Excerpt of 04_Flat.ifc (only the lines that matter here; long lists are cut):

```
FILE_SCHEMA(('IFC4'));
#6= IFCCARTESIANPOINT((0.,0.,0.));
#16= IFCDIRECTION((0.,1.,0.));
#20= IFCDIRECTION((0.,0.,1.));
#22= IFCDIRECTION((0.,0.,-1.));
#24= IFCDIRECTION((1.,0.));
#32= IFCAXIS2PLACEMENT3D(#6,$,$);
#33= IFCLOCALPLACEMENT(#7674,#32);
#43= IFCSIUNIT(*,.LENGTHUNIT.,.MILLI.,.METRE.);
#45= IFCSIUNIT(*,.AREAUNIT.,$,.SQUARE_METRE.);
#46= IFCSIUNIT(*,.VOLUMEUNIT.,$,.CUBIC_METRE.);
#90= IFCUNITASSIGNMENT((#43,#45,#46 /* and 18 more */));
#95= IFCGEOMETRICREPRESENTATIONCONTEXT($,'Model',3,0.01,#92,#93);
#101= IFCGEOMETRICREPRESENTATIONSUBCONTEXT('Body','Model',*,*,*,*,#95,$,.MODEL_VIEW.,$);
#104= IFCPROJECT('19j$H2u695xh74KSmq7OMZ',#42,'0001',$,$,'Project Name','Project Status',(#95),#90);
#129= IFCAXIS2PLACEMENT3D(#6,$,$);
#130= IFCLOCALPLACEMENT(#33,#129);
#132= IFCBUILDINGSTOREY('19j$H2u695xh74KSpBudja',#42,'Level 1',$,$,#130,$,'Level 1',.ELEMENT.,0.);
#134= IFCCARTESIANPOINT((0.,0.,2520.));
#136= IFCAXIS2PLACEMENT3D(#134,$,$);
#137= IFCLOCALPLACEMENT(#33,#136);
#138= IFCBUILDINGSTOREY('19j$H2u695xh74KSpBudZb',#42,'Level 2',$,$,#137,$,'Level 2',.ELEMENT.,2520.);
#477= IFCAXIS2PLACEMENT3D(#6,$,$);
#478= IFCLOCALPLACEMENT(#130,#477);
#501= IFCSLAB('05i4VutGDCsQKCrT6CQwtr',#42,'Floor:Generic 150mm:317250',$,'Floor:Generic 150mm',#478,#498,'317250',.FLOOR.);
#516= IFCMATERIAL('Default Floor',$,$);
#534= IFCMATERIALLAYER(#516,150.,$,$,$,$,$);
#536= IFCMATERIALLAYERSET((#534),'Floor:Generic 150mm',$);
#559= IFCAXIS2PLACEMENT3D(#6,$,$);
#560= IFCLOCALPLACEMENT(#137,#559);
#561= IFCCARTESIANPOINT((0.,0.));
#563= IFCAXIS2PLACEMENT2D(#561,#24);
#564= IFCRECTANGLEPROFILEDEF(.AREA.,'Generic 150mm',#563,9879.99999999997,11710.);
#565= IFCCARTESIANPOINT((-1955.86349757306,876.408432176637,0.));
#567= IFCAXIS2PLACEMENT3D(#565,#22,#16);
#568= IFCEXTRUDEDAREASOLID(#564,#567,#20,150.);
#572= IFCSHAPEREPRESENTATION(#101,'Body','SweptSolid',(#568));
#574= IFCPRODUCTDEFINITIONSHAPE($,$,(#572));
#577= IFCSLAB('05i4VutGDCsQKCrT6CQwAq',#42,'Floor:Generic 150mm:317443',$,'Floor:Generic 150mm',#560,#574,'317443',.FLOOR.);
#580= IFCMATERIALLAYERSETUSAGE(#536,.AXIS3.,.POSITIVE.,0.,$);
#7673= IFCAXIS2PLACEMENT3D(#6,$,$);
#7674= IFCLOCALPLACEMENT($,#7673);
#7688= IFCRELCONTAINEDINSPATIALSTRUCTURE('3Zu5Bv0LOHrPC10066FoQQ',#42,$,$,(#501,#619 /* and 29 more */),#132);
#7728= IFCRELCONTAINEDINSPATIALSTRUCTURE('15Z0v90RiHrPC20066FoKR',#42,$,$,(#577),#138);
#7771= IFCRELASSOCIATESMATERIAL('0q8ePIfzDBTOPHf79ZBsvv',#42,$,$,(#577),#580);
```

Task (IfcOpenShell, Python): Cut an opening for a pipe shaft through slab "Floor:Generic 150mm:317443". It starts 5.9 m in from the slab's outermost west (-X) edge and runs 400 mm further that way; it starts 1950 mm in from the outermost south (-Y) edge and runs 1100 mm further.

```python
import numpy as np
import ifcopenshell
import ifcopenshell.api.feature
import ifcopenshell.api.geometry
import ifcopenshell.api.root
import ifcopenshell.geom
import ifcopenshell.util.placement
import ifcopenshell.util.representation
import ifcopenshell.util.shape
import ifcopenshell.util.unit

model = ifcopenshell.open("04_Flat.ifc")
unit_scale = ifcopenshell.util.unit.calculate_unit_scale(model)
settings = ifcopenshell.geom.settings()


def volume(element):
    """Net volume in cubic metres, openings subtracted."""
    shape = ifcopenshell.geom.create_shape(settings, element)
    return ifcopenshell.util.shape.get_volume(shape.geometry)


slab = model.by_guid("05i4VutGDCsQKCrT6CQwAq")
before = volume(slab)

# Extent in the slab's own axes, in metres. The edges named are its -X and -Y sides.
slab_shape = ifcopenshell.geom.create_shape(settings, slab)
vertices = ifcopenshell.util.shape.get_vertices(slab_shape.geometry)
x_min, y_min, bottom = vertices.min(axis=0)
top = vertices[:, 2].max()

opening = ifcopenshell.api.root.create_entity(model, ifc_class="IfcOpeningElement", name="Pipe shaft opening", predefined_type="OPENING")
context = ifcopenshell.util.representation.get_context(model, "Model", "Body", "MODEL_VIEW")
width, depth = 0.4, 1.1
outline = [(0.0, 0.0), (width, 0.0), (width, depth), (0.0, depth), (0.0, 0.0)]
# Overshoot both faces by 50 mm so the cut is clean.
shape = ifcopenshell.api.geometry.add_slab_representation(
    model, context=context, depth=top - bottom + 0.1, polyline=outline
)
ifcopenshell.api.geometry.assign_representation(model, product=opening, representation=shape)

matrix = ifcopenshell.util.placement.get_local_placement(slab.ObjectPlacement)
matrix[:, 3] = matrix @ np.append(np.array([x_min + 5.9, y_min + 1.95, bottom - 0.05]) / unit_scale, 1.0)
ifcopenshell.api.geometry.edit_object_placement(model, product=opening, matrix=matrix, is_si=False)
ifcopenshell.api.feature.add_feature(model, feature=opening, element=slab)

after = volume(slab)

print(f"slab volume {before:.3f} -> {after:.3f} m3")

model.write("04_Flat_v2.ifc")
```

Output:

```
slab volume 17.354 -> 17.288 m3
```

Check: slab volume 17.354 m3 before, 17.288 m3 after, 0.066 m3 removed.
